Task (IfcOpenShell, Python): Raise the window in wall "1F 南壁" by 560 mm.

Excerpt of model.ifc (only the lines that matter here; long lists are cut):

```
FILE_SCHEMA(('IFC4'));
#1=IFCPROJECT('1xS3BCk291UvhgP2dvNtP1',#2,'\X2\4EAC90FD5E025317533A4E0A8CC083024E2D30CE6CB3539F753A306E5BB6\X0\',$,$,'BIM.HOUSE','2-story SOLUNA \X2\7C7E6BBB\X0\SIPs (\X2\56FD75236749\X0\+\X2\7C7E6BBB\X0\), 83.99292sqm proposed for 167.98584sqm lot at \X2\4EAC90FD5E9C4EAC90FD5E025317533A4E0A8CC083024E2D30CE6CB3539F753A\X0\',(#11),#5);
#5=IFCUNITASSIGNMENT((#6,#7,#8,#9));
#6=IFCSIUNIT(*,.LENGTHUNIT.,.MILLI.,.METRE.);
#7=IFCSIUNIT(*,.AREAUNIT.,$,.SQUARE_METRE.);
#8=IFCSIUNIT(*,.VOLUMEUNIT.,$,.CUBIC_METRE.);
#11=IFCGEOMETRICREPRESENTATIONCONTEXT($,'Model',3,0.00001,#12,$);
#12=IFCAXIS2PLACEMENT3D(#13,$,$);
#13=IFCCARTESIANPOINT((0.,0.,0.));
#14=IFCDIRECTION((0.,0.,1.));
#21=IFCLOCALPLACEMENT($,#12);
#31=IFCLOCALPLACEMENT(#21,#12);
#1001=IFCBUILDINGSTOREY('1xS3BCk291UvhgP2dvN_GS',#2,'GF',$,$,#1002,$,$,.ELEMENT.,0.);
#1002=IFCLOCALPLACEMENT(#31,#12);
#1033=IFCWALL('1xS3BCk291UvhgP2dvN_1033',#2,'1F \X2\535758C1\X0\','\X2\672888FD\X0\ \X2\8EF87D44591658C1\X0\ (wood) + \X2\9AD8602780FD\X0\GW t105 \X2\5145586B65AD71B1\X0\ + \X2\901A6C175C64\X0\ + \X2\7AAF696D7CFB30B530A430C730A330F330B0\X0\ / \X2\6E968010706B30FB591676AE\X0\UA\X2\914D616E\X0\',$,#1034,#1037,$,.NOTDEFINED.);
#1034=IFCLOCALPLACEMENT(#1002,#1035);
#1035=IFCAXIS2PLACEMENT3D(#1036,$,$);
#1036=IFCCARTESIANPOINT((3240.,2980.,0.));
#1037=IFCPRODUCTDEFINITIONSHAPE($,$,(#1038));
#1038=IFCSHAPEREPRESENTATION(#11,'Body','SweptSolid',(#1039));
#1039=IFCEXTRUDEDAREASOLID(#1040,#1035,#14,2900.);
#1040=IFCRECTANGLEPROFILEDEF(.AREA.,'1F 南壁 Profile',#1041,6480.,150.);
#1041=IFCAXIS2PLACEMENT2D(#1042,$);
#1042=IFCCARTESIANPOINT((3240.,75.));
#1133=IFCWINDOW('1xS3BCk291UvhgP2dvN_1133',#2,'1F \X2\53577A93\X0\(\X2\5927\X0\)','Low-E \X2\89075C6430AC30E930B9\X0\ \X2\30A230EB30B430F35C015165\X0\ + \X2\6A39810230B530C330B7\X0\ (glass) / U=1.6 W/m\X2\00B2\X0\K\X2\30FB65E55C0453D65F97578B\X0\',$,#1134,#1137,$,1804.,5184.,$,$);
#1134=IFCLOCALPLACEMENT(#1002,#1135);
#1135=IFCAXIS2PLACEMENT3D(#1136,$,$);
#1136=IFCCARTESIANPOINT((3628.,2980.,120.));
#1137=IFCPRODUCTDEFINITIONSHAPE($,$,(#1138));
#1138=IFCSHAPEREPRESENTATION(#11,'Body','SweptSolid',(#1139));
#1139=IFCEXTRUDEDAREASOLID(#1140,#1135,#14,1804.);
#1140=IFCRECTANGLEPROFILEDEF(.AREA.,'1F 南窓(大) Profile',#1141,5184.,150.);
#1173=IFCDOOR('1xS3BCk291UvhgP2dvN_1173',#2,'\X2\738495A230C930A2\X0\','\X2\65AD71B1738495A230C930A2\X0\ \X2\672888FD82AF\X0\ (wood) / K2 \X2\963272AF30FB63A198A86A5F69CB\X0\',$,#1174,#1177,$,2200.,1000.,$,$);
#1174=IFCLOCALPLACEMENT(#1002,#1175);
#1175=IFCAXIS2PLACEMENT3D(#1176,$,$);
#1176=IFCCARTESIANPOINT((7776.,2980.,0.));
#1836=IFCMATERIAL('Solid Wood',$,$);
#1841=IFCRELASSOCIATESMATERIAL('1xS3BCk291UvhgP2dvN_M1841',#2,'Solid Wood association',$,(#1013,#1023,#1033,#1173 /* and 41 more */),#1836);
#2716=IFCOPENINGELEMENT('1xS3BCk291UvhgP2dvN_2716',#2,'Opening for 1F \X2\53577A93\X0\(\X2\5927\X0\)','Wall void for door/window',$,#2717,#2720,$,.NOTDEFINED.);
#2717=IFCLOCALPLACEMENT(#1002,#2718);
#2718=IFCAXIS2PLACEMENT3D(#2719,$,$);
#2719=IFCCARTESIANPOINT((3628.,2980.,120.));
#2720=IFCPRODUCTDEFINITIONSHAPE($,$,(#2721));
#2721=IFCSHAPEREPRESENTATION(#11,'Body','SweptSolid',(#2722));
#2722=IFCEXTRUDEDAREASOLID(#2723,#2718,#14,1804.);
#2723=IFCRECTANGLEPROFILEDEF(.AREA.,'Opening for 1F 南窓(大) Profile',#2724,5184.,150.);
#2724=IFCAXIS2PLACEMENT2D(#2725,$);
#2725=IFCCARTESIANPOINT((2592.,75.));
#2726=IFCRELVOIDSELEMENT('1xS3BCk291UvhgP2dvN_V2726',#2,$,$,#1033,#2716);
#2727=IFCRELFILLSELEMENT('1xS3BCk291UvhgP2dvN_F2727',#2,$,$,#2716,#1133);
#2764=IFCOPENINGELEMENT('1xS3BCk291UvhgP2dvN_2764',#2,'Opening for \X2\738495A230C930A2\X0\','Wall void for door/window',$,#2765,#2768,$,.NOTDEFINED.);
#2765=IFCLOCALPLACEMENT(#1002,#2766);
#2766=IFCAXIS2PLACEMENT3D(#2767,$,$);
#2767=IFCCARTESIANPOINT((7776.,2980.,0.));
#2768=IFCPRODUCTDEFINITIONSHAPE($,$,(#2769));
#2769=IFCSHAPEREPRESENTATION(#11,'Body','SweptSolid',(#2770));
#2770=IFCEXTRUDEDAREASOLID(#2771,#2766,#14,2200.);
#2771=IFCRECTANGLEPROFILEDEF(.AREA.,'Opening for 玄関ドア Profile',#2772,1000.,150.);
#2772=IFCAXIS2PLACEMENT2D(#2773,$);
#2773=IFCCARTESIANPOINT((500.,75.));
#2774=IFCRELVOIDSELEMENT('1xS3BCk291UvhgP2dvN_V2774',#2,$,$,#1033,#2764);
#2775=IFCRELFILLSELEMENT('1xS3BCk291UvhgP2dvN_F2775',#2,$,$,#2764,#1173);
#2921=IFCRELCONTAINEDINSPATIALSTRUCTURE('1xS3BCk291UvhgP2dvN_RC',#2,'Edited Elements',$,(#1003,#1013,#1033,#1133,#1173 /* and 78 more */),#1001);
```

```python
import numpy as np
import ifcopenshell
import ifcopenshell.api.geometry
import ifcopenshell.util.placement
import ifcopenshell.util.unit

model = ifcopenshell.open("model.ifc")
unit_scale = ifcopenshell.util.unit.calculate_unit_scale(model)

window = model.by_id(1133)
opening = window.FillsVoids[0].RelatingOpeningElement
dz = 560.0

shift = np.array([0.0, 0.0, dz])
# The window is not placed relative to its opening, so move both.
for product in (opening, window):
    matrix = ifcopenshell.util.placement.get_local_placement(product.ObjectPlacement)
    matrix[:3, 3] += shift
    ifcopenshell.api.geometry.edit_object_placement(model, product=product, matrix=matrix, is_si=False)

print(f"moved by {dz * unit_scale:+.3f} m")

model.write("model_v2.ifc")
```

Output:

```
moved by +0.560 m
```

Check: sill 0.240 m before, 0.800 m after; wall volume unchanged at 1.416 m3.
